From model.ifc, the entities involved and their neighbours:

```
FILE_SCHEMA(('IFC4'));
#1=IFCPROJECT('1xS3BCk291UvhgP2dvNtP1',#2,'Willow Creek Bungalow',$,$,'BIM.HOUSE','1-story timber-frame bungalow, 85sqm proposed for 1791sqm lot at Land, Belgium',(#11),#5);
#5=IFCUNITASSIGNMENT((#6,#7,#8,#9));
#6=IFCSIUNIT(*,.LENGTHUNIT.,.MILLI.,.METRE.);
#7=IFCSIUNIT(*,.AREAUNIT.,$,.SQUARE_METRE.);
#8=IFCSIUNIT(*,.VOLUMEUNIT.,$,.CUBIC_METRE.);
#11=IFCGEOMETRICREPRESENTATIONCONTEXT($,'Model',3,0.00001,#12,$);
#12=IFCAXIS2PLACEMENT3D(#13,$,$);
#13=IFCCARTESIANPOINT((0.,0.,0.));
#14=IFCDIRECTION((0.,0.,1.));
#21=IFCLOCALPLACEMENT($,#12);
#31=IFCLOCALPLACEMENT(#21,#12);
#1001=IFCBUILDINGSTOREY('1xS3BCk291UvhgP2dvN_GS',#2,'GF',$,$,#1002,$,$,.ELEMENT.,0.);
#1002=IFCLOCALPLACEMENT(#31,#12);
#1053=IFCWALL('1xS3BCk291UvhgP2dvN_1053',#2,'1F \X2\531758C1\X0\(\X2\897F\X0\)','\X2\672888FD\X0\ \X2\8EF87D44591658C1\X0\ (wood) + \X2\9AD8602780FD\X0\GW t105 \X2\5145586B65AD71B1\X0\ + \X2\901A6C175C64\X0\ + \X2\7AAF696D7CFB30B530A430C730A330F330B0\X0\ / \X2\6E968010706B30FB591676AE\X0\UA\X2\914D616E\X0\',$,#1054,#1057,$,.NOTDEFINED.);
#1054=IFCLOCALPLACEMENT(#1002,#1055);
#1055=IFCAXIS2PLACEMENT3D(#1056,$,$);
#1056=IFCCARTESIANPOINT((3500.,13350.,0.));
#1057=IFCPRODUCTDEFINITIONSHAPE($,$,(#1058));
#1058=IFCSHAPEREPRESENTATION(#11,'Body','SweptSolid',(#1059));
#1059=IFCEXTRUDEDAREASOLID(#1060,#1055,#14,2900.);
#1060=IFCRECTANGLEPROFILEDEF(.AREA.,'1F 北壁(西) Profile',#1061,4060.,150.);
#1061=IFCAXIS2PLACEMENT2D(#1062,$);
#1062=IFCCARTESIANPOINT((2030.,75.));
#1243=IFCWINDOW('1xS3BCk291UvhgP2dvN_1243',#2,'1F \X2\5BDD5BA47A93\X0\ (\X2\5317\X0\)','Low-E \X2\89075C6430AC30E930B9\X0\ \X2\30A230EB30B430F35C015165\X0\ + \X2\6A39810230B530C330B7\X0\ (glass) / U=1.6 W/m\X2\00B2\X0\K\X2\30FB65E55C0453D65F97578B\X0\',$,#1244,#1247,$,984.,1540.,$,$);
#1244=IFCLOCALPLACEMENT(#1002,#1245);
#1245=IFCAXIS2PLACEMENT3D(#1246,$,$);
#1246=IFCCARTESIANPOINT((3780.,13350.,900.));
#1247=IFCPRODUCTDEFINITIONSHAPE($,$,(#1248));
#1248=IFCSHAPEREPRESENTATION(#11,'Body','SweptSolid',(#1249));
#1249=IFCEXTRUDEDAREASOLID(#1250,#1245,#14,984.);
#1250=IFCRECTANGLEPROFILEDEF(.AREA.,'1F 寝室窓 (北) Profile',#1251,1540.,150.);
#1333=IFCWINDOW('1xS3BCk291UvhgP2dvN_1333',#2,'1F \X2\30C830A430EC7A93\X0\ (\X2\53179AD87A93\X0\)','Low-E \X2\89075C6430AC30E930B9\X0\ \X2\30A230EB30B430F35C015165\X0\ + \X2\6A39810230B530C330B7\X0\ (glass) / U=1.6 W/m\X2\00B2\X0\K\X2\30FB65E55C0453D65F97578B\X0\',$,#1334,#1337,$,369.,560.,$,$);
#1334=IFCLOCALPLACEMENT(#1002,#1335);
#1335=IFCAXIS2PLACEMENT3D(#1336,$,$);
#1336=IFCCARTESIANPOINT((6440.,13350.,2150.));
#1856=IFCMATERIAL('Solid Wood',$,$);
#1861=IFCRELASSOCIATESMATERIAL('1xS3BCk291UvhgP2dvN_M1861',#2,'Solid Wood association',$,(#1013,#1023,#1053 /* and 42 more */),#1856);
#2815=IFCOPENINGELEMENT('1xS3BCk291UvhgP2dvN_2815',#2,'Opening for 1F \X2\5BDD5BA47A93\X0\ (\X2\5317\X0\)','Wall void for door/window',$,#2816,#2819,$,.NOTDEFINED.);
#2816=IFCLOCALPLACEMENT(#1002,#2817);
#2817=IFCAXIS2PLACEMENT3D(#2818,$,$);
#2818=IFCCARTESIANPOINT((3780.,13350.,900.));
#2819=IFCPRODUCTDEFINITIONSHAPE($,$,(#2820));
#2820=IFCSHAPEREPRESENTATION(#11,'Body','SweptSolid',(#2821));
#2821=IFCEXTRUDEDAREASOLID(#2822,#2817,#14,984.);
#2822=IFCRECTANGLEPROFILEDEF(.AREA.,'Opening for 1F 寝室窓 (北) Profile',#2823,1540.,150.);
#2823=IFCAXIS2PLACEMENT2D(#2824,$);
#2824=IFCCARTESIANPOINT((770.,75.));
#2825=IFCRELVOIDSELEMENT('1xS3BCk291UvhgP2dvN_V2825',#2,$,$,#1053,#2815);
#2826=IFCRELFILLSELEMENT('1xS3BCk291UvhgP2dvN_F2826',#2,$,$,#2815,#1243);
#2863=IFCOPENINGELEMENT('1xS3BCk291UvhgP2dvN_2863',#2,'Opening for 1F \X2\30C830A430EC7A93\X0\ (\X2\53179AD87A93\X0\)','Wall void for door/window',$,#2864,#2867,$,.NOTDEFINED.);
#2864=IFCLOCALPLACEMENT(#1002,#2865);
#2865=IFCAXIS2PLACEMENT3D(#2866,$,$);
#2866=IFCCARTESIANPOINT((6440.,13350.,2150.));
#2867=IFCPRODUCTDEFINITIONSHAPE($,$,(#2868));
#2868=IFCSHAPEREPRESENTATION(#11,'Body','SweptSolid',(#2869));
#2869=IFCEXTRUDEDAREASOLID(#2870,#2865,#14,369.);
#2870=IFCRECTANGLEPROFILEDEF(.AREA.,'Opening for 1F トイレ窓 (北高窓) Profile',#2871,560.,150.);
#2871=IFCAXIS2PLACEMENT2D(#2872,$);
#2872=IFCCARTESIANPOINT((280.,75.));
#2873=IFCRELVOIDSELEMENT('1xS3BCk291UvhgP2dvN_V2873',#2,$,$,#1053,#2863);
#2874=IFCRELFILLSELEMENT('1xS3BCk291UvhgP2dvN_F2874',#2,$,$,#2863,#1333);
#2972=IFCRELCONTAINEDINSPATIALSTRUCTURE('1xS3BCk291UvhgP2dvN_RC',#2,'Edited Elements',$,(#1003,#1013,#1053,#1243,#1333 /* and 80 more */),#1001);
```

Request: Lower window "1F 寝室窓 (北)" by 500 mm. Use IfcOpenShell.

```python
import numpy as np
import ifcopenshell
import ifcopenshell.api.geometry
import ifcopenshell.util.placement
import ifcopenshell.util.unit

model = ifcopenshell.open("model.ifc")
unit_scale = ifcopenshell.util.unit.calculate_unit_scale(model)

window = model.by_guid("1xS3BCk291UvhgP2dvN_1243")
opening = window.FillsVoids[0].RelatingOpeningElement
dz = -0.5 / unit_scale

shift = np.array([0.0, 0.0, dz])
# The window is not placed relative to its opening, so move both.
for product in (opening, window):
    matrix = ifcopenshell.util.placement.get_local_placement(product.ObjectPlacement)
    matrix[:3, 3] += shift
    ifcopenshell.api.geometry.edit_object_placement(model, product=product, matrix=matrix, is_si=False)

print(f"moved by {dz * unit_scale:+.3f} m")

model.write("model_edited.ifc")
```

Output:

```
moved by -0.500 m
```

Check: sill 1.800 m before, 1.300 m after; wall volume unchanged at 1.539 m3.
